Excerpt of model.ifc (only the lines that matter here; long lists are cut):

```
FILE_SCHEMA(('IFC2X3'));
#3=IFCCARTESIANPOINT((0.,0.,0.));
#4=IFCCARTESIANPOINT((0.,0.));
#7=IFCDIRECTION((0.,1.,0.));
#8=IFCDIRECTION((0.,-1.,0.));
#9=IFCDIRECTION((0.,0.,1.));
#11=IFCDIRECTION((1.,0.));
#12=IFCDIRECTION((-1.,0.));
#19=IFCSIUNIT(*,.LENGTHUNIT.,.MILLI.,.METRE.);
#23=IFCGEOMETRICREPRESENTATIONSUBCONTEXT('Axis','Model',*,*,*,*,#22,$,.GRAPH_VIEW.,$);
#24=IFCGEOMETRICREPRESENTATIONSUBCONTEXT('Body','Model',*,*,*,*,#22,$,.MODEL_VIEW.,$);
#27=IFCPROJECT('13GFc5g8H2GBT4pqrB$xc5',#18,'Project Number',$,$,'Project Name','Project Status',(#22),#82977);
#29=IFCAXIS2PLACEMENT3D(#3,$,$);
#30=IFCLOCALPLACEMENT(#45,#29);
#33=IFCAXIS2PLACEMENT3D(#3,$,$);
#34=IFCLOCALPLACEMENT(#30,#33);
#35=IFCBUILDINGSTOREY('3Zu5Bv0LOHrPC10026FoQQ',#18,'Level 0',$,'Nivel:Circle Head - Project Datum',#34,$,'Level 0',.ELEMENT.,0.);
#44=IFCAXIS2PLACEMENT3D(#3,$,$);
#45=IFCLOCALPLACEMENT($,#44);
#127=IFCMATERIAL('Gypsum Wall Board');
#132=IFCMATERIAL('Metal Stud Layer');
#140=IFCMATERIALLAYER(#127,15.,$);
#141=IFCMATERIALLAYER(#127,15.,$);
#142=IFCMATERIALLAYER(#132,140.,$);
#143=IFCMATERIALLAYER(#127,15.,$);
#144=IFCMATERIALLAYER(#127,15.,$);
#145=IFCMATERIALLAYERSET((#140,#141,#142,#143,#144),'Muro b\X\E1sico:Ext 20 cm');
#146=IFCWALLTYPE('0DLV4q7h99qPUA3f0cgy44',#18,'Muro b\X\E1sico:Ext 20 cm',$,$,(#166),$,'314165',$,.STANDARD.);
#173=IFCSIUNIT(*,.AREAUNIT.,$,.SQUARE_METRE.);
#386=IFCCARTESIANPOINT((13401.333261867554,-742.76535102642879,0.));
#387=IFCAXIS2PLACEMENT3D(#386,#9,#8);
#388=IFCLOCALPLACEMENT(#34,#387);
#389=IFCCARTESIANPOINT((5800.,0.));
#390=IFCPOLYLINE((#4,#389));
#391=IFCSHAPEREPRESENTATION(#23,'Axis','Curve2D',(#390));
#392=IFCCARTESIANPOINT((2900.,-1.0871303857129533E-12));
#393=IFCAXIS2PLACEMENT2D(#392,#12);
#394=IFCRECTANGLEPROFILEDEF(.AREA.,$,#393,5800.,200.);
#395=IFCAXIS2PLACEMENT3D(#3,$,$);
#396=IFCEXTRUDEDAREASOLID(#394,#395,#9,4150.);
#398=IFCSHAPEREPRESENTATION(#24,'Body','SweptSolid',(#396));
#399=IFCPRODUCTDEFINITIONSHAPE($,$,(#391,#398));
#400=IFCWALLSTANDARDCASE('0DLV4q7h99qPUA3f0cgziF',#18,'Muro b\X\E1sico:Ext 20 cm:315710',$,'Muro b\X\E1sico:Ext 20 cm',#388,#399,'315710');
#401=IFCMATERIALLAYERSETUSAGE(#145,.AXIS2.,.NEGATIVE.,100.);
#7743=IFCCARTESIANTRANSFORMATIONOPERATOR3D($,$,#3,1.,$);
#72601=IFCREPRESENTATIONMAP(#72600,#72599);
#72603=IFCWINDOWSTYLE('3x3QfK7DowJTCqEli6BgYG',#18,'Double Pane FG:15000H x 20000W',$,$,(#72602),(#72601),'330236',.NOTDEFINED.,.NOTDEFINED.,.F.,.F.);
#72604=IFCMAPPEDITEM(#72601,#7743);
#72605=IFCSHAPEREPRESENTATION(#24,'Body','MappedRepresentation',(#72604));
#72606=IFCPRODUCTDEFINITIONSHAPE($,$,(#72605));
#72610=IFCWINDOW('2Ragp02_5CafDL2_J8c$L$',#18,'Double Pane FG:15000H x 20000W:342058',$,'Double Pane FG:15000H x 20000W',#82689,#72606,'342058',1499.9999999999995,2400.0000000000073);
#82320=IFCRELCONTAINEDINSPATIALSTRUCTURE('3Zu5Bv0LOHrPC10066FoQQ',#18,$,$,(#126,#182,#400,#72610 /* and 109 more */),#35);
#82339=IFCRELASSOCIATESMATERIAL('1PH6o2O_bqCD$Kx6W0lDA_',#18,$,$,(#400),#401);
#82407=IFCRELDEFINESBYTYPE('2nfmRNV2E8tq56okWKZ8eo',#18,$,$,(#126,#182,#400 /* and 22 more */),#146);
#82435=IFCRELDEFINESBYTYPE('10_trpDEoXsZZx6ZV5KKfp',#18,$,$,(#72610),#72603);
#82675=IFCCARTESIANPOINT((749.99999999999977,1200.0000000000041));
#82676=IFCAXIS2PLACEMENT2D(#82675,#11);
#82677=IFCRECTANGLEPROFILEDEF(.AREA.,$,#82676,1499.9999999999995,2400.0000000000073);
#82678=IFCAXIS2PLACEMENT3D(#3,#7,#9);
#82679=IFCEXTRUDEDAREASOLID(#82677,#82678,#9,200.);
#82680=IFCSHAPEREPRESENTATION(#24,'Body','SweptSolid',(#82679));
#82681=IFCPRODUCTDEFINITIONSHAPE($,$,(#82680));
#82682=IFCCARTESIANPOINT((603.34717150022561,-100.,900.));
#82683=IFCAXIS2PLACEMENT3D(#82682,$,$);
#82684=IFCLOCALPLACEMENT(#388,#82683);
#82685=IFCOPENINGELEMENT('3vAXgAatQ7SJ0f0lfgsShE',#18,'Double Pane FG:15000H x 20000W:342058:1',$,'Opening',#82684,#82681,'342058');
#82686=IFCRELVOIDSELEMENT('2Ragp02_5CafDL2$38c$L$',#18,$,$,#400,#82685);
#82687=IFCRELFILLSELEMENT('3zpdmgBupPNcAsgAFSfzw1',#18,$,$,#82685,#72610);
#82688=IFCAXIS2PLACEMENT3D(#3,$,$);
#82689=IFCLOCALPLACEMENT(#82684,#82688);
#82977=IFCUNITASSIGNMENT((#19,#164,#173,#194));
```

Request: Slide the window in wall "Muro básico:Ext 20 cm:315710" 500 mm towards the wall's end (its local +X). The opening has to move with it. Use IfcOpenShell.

```python
import ifcopenshell
import ifcopenshell.api.geometry
import ifcopenshell.util.placement
import ifcopenshell.util.unit

model = ifcopenshell.open("model.ifc")
unit_scale = ifcopenshell.util.unit.calculate_unit_scale(model)

window = model.by_guid("2Ragp02_5CafDL2_J8c$L$")
opening = window.FillsVoids[0].RelatingOpeningElement
wall = opening.VoidsElements[0].RelatingBuildingElement

wall_matrix = ifcopenshell.util.placement.get_local_placement(wall.ObjectPlacement)
shift = wall_matrix[:3, 0] * 0.5 / unit_scale
before = ifcopenshell.util.placement.get_local_placement(window.ObjectPlacement)[:3, 3].copy()

# The window is placed relative to its opening, so it follows when the opening moves.
matrix = ifcopenshell.util.placement.get_local_placement(opening.ObjectPlacement)
matrix[:3, 3] += shift
ifcopenshell.api.geometry.edit_object_placement(
    model, product=opening, matrix=matrix, is_si=False, should_transform_children=True
)

after = ifcopenshell.util.placement.get_local_placement(window.ObjectPlacement)[:3, 3]
print("window moved by", (after - before).round(3) + 0.0)

model.write("model-out.ifc")
```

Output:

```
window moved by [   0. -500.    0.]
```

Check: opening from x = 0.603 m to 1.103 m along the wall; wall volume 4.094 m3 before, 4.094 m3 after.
